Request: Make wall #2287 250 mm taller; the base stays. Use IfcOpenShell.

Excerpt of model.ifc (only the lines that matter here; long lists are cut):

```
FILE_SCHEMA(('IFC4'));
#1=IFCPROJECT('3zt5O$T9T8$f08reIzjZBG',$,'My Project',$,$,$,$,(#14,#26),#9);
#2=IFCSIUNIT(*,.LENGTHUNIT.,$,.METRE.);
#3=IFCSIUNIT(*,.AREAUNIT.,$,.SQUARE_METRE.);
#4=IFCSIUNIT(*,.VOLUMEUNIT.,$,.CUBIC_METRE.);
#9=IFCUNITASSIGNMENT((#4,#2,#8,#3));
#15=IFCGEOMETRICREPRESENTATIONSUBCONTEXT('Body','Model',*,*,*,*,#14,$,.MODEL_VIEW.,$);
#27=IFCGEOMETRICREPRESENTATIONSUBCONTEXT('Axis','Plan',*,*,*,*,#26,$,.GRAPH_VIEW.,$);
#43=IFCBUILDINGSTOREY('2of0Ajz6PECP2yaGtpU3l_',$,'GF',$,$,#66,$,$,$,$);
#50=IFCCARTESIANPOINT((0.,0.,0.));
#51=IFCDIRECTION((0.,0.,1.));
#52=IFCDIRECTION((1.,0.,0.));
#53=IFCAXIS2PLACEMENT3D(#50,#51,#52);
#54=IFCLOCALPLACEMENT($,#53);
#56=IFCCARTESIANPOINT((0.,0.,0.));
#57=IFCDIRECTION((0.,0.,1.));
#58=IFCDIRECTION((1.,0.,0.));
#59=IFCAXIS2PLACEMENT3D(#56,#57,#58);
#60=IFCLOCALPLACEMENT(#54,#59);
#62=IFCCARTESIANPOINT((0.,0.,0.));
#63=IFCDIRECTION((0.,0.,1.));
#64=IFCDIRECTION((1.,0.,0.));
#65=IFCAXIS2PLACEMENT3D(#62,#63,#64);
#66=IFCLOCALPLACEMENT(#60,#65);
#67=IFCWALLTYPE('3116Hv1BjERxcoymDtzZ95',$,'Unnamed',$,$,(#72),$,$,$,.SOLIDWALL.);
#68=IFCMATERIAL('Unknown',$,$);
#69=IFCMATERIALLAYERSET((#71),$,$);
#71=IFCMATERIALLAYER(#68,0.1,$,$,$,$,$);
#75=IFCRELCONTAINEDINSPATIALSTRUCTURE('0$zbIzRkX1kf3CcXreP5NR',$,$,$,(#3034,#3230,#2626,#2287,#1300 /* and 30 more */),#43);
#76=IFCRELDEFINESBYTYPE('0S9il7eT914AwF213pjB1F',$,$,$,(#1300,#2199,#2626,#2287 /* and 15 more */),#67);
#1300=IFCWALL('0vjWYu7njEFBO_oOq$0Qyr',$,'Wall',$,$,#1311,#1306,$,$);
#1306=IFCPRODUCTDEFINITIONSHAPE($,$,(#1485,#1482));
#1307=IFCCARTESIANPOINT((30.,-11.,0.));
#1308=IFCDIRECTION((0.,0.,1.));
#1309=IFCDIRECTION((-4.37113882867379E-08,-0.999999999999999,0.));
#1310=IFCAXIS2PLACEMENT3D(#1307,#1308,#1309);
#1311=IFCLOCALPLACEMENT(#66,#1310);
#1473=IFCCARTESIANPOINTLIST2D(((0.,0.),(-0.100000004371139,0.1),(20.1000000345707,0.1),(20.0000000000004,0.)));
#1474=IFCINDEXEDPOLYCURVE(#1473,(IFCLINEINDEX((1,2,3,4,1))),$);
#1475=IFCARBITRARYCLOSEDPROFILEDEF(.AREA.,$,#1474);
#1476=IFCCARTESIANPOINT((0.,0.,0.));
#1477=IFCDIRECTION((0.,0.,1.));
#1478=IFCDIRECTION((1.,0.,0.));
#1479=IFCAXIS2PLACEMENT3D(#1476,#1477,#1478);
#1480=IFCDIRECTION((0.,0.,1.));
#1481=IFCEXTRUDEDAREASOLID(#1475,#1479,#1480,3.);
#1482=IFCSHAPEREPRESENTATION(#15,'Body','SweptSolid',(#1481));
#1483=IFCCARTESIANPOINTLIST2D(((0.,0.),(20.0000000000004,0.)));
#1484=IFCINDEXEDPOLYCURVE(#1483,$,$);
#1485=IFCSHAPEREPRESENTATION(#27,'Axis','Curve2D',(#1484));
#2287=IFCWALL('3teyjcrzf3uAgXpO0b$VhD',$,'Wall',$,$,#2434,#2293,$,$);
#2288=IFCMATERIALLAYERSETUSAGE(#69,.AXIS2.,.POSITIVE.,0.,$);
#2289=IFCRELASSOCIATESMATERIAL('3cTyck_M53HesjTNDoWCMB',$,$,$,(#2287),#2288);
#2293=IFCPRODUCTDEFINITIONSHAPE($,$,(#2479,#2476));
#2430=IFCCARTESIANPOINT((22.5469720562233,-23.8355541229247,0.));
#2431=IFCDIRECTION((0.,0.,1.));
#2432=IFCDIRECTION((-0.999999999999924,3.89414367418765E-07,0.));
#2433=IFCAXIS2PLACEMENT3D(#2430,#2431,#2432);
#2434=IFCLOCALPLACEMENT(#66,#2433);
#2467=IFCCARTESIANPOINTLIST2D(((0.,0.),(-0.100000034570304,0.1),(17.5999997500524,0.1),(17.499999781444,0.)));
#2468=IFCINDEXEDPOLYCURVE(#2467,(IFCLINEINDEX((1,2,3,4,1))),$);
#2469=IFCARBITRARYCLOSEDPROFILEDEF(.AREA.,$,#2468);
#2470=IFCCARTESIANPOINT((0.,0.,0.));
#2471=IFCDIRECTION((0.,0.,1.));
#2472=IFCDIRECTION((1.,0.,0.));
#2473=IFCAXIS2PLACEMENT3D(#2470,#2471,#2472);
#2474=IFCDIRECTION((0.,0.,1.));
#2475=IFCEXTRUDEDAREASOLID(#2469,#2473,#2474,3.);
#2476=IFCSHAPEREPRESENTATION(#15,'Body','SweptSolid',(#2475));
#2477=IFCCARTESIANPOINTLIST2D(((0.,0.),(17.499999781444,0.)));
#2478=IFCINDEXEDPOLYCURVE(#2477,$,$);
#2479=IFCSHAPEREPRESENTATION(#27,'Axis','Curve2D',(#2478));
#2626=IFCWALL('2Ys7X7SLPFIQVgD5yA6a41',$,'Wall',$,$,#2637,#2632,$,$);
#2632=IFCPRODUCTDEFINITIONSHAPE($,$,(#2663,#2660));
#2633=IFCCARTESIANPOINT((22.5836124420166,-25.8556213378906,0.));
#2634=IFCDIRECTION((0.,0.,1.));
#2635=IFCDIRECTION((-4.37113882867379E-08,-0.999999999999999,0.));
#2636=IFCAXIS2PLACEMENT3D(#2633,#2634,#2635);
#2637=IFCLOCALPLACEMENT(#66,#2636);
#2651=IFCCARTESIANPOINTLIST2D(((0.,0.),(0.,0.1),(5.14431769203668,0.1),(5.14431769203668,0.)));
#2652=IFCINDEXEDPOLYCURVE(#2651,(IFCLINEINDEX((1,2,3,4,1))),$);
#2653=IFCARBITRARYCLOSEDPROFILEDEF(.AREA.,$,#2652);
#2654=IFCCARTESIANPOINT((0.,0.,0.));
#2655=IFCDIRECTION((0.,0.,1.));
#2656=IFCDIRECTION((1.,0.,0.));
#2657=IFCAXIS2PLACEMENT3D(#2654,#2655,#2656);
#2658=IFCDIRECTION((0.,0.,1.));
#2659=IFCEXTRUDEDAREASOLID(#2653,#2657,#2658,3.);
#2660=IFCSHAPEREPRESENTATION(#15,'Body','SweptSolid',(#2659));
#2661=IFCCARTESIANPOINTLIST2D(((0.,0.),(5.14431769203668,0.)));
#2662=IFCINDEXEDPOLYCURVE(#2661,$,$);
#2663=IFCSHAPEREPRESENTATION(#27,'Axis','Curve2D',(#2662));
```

```python
import ifcopenshell
import ifcopenshell.geom
import ifcopenshell.util.representation
import ifcopenshell.util.shape

model = ifcopenshell.open("model.ifc")
settings = ifcopenshell.geom.settings()


def volume(element):
    """Net volume in cubic metres, openings subtracted."""
    shape = ifcopenshell.geom.create_shape(settings, element)
    return ifcopenshell.util.shape.get_volume(shape.geometry)


wall = model.by_guid("3teyjcrzf3uAgXpO0b$VhD")
before = volume(wall)

body = ifcopenshell.util.representation.get_representation(wall, "Model", "Body")
solid = body.Items[0]
old_height = solid.Depth
solid.Depth += 0.25
after = volume(wall)

print(f"height {old_height:g} -> {solid.Depth:g}, volume {before:.3f} -> {after:.3f} m3")

model.write("model-out.ifc")
```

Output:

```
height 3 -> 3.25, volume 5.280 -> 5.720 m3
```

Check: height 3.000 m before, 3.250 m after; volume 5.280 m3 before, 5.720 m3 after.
